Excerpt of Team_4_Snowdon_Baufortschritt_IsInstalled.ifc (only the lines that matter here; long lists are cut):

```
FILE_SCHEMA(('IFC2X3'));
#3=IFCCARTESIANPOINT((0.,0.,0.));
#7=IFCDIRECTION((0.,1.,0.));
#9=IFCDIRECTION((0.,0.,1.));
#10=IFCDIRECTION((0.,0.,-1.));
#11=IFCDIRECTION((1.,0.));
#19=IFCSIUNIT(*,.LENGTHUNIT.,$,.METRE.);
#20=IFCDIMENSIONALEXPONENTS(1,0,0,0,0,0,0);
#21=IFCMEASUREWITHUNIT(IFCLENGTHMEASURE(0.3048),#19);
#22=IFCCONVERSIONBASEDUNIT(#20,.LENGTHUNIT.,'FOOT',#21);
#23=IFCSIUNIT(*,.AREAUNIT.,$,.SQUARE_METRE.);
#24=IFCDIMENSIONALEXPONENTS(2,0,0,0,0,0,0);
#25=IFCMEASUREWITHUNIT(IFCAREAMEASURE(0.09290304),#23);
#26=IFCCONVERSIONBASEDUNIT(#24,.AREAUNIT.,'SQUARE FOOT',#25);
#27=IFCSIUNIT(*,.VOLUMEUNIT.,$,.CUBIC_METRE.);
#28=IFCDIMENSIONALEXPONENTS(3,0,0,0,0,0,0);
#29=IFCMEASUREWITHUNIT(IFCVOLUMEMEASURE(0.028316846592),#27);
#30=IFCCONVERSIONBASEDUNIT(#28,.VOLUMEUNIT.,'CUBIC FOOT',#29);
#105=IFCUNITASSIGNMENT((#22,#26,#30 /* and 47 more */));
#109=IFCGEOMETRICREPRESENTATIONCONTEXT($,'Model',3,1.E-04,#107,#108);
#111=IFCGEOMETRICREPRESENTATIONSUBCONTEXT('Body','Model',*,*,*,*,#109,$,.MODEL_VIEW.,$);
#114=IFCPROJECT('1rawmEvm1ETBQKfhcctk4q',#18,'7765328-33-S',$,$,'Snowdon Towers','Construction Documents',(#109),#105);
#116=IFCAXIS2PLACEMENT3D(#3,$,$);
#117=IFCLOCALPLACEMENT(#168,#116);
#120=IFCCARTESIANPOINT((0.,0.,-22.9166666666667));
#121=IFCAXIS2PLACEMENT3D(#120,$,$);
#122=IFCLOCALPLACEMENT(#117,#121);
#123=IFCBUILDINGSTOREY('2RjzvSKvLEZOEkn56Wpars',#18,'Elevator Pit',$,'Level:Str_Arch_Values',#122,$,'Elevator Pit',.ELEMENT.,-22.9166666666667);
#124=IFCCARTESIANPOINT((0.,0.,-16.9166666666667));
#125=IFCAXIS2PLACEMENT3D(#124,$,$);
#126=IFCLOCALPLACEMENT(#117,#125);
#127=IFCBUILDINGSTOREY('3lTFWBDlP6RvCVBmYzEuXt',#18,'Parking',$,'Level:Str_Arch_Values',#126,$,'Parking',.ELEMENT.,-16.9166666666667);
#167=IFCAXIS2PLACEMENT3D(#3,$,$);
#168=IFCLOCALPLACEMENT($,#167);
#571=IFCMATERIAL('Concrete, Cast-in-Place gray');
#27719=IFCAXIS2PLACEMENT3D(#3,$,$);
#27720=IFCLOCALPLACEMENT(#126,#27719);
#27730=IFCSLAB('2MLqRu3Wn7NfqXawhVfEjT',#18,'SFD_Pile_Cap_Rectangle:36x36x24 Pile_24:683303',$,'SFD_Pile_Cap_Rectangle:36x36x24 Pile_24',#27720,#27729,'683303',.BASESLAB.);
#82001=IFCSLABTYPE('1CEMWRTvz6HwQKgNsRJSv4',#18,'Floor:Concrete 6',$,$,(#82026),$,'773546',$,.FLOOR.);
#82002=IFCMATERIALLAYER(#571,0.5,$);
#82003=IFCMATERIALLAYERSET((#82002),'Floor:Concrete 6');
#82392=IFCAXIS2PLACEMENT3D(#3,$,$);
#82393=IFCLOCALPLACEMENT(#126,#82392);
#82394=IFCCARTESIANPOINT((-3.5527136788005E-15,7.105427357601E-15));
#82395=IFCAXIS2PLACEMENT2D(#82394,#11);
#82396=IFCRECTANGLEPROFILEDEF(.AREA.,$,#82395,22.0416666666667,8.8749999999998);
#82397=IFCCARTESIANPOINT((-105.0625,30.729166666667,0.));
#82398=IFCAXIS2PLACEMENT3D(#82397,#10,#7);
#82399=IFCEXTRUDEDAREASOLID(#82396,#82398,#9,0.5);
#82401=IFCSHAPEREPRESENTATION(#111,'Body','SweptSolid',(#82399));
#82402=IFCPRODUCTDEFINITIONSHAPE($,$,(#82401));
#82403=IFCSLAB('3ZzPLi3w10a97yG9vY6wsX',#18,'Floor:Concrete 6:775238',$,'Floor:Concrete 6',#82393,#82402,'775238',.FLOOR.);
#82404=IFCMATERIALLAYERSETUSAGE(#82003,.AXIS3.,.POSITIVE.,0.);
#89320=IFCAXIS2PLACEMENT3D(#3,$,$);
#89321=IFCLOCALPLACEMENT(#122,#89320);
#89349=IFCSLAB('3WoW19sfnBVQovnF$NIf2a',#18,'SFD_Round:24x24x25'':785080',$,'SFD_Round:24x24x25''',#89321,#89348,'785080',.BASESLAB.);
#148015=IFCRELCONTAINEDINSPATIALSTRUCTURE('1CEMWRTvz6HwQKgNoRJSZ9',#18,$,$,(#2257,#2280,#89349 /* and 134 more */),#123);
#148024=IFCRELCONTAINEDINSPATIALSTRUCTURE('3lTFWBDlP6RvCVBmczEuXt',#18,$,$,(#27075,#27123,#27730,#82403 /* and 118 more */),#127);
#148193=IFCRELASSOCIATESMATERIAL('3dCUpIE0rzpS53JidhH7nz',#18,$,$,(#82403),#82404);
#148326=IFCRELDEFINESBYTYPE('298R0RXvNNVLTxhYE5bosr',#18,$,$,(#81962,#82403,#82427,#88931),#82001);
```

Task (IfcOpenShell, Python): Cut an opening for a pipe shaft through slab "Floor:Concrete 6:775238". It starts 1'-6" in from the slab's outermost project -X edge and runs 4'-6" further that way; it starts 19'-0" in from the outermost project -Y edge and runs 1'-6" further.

```python
import numpy as np
import ifcopenshell
import ifcopenshell.api.feature
import ifcopenshell.api.geometry
import ifcopenshell.api.root
import ifcopenshell.geom
import ifcopenshell.util.placement
import ifcopenshell.util.representation
import ifcopenshell.util.shape
import ifcopenshell.util.unit

model = ifcopenshell.open("Team_4_Snowdon_Baufortschritt_IsInstalled.ifc")
unit_scale = ifcopenshell.util.unit.calculate_unit_scale(model)
settings = ifcopenshell.geom.settings()


def volume(element):
    """Net volume in cubic metres, openings subtracted."""
    shape = ifcopenshell.geom.create_shape(settings, element)
    return ifcopenshell.util.shape.get_volume(shape.geometry)


slab = model.by_guid("3ZzPLi3w10a97yG9vY6wsX")
before = volume(slab)

# Extent in the slab's own axes, in metres. The edges named are its -X and -Y sides.
slab_shape = ifcopenshell.geom.create_shape(settings, slab)
vertices = ifcopenshell.util.shape.get_vertices(slab_shape.geometry)
x_min, y_min, bottom = vertices.min(axis=0)
top = vertices[:, 2].max()

opening = ifcopenshell.api.root.create_entity(model, ifc_class="IfcOpeningElement", name="Pipe shaft opening")
context = ifcopenshell.util.representation.get_context(model, "Model", "Body", "MODEL_VIEW")
width, depth = 1.3716, 0.4572
outline = [(0.0, 0.0), (width, 0.0), (width, depth), (0.0, depth), (0.0, 0.0)]
# Overshoot both faces by 50 mm so the cut is clean.
shape = ifcopenshell.api.geometry.add_slab_representation(
    model, context=context, depth=top - bottom + 0.1, polyline=outline
)
ifcopenshell.api.geometry.assign_representation(model, product=opening, representation=shape)

matrix = ifcopenshell.util.placement.get_local_placement(slab.ObjectPlacement)
matrix[:, 3] = matrix @ np.append(np.array([x_min + 0.4572, y_min + 5.7912, bottom - 0.05]) / unit_scale, 1.0)
ifcopenshell.api.geometry.edit_object_placement(model, product=opening, matrix=matrix, is_si=False)
ifcopenshell.api.feature.add_feature(model, feature=opening, element=slab)

after = volume(slab)

print(f"slab volume {before:.3f} -> {after:.3f} m3")

model.write("Team_4_Snowdon_Baufortschritt_IsInstalled_updated.ifc")
```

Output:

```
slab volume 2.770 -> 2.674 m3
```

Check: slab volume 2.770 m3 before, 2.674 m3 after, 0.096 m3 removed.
